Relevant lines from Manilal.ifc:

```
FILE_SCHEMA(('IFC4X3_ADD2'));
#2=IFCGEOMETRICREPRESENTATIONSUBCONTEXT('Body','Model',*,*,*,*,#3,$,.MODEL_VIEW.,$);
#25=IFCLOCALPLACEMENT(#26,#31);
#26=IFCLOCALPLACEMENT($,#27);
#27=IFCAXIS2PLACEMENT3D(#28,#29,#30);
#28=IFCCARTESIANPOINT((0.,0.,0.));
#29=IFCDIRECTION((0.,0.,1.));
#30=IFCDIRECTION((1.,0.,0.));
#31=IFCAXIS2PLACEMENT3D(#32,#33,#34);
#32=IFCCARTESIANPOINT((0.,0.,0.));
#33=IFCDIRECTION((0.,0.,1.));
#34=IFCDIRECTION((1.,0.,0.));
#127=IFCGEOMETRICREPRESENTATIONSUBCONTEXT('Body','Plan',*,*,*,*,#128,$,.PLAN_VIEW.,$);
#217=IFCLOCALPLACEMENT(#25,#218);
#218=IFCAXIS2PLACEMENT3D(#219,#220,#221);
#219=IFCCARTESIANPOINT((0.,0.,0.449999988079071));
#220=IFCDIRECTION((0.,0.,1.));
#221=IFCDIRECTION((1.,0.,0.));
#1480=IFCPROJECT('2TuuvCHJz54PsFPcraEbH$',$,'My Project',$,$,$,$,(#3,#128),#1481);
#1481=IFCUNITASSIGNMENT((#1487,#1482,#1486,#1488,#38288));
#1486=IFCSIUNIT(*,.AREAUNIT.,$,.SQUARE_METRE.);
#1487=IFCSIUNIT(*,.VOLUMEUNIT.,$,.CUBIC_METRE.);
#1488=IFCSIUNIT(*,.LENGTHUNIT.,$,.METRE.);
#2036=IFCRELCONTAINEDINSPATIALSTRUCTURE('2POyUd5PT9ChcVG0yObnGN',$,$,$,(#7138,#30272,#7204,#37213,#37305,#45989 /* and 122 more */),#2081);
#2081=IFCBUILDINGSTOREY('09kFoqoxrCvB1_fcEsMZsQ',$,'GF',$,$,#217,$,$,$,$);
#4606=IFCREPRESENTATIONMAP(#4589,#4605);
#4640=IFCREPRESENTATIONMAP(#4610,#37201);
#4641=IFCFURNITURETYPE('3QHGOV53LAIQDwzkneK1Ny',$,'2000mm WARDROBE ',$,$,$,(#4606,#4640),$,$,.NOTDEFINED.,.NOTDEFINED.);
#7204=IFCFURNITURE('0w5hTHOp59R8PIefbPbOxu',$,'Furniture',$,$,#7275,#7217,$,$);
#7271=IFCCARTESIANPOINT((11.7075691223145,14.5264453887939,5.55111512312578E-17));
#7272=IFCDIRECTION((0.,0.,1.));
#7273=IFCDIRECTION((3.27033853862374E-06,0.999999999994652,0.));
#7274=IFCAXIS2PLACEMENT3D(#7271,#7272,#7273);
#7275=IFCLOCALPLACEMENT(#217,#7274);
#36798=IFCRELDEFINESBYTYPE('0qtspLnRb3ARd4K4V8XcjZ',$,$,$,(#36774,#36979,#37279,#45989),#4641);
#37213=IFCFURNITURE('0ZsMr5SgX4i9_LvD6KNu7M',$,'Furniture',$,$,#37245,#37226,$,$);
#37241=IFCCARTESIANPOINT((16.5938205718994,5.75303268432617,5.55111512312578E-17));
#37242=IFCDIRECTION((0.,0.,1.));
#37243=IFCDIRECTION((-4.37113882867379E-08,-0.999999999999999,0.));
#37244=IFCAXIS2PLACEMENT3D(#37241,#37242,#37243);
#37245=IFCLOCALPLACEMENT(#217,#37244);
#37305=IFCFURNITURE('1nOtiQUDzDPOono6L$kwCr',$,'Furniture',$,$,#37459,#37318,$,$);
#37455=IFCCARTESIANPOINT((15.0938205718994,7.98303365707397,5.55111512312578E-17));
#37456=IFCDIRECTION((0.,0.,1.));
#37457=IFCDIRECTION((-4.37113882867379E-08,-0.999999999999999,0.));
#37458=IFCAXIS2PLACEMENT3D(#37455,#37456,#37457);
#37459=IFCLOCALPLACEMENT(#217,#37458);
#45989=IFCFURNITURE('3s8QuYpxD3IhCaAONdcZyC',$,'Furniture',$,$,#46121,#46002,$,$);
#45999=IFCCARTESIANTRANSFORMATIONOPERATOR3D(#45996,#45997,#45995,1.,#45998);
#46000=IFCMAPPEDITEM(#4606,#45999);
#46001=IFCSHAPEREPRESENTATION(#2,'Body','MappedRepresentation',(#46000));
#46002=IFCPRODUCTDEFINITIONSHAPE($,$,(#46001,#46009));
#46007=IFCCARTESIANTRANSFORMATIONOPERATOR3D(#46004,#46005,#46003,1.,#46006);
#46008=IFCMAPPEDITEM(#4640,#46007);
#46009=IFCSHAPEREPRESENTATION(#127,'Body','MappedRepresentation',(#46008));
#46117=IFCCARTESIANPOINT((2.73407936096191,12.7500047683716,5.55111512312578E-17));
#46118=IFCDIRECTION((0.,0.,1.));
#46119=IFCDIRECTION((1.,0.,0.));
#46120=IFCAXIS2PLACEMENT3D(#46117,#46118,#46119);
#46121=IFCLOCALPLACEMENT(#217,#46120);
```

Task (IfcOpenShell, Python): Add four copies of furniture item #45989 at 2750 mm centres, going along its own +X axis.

```python
import ifcopenshell
import ifcopenshell.api.geometry
import ifcopenshell.api.root
import ifcopenshell.util.element
import ifcopenshell.util.placement
import ifcopenshell.util.unit

model = ifcopenshell.open("Manilal.ifc")
unit_scale = ifcopenshell.util.unit.calculate_unit_scale(model)

source = model.by_id(45989)
base = ifcopenshell.util.placement.get_local_placement(source.ObjectPlacement)
step = base[:3, 0] * 2.75 / unit_scale

for i in range(1, 5):
    copy = ifcopenshell.api.root.copy_class(model, product=source)
    copy.Representation = ifcopenshell.util.element.copy_deep(
        model, source.Representation, exclude=["IfcGeometricRepresentationContext", "IfcRepresentationMap"]
    )
    matrix = base.copy()
    matrix[:3, 3] += i * step
    print("added at", matrix[:3, 3].round(3) + 0.0)
    ifcopenshell.api.geometry.edit_object_placement(model, product=copy, matrix=matrix, is_si=False)

model.write("Manilal-out.ifc")
```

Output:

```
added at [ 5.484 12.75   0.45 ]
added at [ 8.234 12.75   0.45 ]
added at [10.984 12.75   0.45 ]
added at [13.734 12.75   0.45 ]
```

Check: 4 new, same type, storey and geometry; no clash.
